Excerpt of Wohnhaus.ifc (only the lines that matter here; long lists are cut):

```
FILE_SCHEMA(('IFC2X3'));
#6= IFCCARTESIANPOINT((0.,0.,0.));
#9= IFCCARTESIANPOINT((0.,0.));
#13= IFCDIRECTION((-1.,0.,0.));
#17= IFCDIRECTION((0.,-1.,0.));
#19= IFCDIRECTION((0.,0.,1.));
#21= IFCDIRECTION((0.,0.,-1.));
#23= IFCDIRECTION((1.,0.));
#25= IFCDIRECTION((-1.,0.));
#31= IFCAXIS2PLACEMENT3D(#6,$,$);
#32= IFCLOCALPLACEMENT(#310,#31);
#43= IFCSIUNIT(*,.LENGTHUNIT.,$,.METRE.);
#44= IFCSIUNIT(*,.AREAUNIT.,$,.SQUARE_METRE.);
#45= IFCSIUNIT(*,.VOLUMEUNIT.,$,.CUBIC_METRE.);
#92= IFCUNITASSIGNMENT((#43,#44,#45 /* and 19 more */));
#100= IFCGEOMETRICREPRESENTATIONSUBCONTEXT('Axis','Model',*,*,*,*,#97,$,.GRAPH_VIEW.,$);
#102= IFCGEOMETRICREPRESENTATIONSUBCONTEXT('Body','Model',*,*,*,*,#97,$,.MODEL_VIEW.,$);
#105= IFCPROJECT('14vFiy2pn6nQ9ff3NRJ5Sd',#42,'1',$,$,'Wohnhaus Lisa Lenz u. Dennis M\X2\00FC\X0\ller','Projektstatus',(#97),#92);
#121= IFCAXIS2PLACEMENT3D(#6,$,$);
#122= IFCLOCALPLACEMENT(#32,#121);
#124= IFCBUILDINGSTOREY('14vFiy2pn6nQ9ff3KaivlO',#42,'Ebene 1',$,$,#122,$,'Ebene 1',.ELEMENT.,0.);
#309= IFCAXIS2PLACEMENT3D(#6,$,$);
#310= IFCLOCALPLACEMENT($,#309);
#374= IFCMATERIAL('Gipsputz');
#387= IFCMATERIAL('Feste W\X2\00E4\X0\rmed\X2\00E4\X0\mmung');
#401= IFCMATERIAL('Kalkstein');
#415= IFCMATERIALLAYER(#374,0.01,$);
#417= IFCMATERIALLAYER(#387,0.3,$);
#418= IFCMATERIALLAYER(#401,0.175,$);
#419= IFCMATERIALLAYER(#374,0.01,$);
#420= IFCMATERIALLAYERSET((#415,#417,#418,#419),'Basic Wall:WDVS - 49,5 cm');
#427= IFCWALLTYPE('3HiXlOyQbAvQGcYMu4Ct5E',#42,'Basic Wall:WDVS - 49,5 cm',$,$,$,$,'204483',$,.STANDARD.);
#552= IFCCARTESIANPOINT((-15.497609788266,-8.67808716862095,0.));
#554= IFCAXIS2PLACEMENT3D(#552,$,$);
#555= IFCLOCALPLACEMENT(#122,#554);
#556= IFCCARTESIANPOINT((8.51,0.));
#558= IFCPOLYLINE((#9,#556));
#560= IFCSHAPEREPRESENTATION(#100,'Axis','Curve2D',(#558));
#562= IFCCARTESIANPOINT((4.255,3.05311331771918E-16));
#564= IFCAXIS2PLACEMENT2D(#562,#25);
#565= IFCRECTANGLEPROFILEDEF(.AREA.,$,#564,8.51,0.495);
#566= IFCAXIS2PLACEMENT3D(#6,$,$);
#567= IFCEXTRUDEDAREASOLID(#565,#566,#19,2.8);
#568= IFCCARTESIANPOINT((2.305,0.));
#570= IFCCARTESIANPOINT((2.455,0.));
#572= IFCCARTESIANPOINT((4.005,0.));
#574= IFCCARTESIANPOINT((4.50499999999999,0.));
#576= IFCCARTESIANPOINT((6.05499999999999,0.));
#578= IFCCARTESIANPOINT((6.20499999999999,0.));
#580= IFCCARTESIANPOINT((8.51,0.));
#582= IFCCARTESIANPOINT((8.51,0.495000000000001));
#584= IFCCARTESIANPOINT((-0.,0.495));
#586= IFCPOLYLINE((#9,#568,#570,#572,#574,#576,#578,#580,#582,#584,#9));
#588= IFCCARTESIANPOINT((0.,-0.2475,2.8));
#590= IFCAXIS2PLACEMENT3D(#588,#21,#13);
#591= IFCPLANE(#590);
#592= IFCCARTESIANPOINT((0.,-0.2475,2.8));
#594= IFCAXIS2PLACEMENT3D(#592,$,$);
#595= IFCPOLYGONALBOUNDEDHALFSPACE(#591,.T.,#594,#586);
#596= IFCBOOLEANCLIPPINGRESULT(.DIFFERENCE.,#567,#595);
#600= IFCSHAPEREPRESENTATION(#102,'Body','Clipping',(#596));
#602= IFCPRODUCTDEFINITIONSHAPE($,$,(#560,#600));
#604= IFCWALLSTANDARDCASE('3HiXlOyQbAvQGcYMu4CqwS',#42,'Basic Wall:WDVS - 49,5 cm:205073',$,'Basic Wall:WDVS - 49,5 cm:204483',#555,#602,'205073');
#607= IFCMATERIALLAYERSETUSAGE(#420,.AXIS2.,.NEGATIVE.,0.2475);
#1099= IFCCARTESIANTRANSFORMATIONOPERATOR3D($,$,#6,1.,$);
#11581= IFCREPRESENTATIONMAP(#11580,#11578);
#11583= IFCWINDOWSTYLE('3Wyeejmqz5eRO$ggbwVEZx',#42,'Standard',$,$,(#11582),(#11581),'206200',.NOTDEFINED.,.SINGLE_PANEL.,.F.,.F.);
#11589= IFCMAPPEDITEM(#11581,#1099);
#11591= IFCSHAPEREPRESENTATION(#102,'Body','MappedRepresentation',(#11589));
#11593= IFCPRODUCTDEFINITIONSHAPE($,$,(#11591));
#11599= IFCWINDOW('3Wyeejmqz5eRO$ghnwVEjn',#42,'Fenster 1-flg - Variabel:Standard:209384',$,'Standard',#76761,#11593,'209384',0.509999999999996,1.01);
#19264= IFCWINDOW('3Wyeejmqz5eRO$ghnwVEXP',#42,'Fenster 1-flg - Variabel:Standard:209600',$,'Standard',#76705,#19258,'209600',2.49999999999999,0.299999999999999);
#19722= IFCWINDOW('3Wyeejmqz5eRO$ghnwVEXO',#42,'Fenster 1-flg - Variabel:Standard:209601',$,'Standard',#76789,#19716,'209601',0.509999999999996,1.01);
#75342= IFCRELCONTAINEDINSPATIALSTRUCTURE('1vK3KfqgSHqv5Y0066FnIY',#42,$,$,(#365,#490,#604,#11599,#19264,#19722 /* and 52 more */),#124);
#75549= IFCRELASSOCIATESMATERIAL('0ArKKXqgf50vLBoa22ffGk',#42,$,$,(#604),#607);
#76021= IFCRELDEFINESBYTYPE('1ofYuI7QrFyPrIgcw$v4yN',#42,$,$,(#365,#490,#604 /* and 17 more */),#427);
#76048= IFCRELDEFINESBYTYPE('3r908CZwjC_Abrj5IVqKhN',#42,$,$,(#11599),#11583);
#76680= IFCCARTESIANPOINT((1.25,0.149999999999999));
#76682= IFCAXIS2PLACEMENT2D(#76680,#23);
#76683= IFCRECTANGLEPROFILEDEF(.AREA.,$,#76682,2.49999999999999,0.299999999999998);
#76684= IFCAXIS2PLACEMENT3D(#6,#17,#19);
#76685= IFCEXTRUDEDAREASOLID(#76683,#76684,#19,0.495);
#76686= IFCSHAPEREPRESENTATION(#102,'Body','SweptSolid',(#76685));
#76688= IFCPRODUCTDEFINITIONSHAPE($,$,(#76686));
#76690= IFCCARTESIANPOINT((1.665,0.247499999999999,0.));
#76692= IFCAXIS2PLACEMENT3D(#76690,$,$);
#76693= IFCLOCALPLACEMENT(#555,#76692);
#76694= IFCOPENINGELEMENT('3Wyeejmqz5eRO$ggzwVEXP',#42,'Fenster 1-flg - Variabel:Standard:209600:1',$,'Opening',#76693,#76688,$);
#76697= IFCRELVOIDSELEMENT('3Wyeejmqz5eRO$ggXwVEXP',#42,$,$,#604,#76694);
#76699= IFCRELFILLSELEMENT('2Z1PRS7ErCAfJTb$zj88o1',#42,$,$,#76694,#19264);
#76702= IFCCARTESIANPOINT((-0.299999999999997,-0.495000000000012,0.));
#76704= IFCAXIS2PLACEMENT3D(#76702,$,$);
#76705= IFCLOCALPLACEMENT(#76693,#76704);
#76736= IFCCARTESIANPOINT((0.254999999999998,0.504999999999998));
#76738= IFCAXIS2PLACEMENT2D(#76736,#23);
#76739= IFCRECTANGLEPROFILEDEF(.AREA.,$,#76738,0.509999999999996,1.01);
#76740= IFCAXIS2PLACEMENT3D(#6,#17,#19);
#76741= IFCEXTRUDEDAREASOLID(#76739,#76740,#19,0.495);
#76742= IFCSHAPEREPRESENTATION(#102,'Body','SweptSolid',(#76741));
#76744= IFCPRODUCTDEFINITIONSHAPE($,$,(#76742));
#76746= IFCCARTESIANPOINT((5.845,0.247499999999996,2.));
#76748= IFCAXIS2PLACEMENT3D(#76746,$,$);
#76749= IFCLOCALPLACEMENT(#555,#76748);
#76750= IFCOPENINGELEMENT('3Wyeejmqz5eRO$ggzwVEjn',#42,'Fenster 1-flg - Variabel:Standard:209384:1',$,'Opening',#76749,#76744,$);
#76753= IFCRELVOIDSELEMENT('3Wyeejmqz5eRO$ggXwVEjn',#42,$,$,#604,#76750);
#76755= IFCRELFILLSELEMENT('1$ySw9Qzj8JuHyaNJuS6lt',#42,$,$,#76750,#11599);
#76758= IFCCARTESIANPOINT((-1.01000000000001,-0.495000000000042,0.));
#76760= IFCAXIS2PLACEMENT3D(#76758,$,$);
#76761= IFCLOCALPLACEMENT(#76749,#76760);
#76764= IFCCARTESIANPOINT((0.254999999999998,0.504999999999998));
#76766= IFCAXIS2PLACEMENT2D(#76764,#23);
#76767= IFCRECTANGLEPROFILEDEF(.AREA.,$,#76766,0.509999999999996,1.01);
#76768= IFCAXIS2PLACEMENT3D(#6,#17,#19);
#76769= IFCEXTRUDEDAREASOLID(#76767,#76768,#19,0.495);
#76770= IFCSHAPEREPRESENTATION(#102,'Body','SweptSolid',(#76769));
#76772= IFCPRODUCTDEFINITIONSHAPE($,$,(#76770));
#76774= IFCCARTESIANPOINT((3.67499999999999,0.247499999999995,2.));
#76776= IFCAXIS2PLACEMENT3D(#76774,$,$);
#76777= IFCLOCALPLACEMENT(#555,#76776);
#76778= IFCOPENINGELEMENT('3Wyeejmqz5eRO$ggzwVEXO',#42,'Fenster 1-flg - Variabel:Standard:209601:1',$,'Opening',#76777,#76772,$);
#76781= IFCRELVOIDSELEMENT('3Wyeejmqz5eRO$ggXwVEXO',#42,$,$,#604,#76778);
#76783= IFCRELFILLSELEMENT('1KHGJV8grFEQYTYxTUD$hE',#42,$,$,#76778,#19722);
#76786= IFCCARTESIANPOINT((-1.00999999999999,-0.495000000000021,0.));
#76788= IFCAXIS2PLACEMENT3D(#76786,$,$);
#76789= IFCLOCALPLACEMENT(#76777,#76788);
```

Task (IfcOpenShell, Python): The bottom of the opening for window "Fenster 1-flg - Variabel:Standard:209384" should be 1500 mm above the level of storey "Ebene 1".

```python
import numpy as np
import ifcopenshell
import ifcopenshell.api.geometry
import ifcopenshell.geom
import ifcopenshell.util.element
import ifcopenshell.util.placement
import ifcopenshell.util.shape
import ifcopenshell.util.unit

model = ifcopenshell.open("Wohnhaus.ifc")
unit_scale = ifcopenshell.util.unit.calculate_unit_scale(model)

window = model.by_guid("3Wyeejmqz5eRO$ghnwVEjn")
opening = window.FillsVoids[0].RelatingOpeningElement
storey = ifcopenshell.util.element.get_container(window, ifc_class="IfcBuildingStorey")
level = ifcopenshell.util.placement.get_local_placement(storey.ObjectPlacement)[2, 3]

# The opening's origin need not be at the sill, so measure its lowest point.
shape = ifcopenshell.geom.create_shape(ifcopenshell.geom.settings(), opening)
bottom = ifcopenshell.util.shape.get_shape_bottom_elevation(shape, shape.geometry) / unit_scale
dz = level + 1.5 / unit_scale - bottom

shift = np.array([0.0, 0.0, dz])
# The window is placed relative to its opening, so it follows when the opening moves.
matrix = ifcopenshell.util.placement.get_local_placement(opening.ObjectPlacement)
matrix[:3, 3] += shift
ifcopenshell.api.geometry.edit_object_placement(
    model, product=opening, matrix=matrix, is_si=False, should_transform_children=True
)

print(f"moved by {dz * unit_scale:+.3f} m")

model.write("Wohnhaus_v2.ifc")
```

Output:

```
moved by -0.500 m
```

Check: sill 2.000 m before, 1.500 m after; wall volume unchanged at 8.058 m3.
